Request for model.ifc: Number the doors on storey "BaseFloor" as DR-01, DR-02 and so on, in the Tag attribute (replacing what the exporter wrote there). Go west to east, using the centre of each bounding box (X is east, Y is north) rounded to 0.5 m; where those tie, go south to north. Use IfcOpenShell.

First a look at what the model holds.

```python
import ifcopenshell
import ifcopenshell.util.element
import ifcopenshell.util.placement

model = ifcopenshell.open("model.ifc")
print(model.schema)
storey = next(s for s in model.by_type("IfcBuildingStorey") if s.Name == "BaseFloor")
doors = [e for e in ifcopenshell.util.element.get_decomposition(storey) if e.is_a("IfcDoor")]
for e in sorted(doors, key=lambda e: e.id()):
    origin = ifcopenshell.util.placement.get_local_placement(e.ObjectPlacement)[:3, 3]
    print(e.id(), e.Tag, e.Name, origin.round(2) + 0.0, sep=" | ")
```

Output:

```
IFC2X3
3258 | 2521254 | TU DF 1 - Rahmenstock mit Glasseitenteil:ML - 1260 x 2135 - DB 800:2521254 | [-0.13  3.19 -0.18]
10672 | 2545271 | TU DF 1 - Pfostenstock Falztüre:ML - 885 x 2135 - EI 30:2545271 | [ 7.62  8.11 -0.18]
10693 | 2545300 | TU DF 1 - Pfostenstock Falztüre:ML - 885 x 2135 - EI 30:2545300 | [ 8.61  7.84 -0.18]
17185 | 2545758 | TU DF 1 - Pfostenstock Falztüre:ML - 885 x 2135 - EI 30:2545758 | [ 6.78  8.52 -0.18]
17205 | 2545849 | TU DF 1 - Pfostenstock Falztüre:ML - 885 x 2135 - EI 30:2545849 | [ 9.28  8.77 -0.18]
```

```python
import ifcopenshell
import ifcopenshell.geom
import ifcopenshell.util.element
import ifcopenshell.util.shape

model = ifcopenshell.open("model.ifc")
settings = ifcopenshell.geom.settings()
settings.set("use-world-coords", True)


def centre(element):
    shape = ifcopenshell.geom.create_shape(settings, element)
    return ifcopenshell.util.shape.get_bbox_centroid(shape.geometry)


storey = next(s for s in model.by_type("IfcBuildingStorey") if s.Name == "BaseFloor")
doors = [e for e in ifcopenshell.util.element.get_decomposition(storey) if e.is_a("IfcDoor")]

# Insertion points can sit at a corner or the storey origin, so sort by the geometry (in metres).
centres = {e: centre(e) for e in doors}
doors.sort(key=lambda e: (round(centres[e][0] / 0.5), centres[e][1]))

for i, e in enumerate(doors, start=1):
    number = f"DR-{i:02d}"
    e.Tag = number
    print(e.id(), number)

model.write("model-out.ifc")
```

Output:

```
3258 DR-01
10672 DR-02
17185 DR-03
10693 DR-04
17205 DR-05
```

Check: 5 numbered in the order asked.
